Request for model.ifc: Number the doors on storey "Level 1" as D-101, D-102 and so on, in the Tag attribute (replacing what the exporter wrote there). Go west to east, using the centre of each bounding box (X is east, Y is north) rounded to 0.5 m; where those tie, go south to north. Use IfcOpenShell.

First a look at what the model holds.

```python
import ifcopenshell
import ifcopenshell.util.element
import ifcopenshell.util.placement

model = ifcopenshell.open("model.ifc")
print(model.schema)
storey = next(s for s in model.by_type("IfcBuildingStorey") if s.Name == "Level 1")
doors = [e for e in ifcopenshell.util.element.get_decomposition(storey) if e.is_a("IfcDoor")]
for e in sorted(doors, key=lambda e: e.id()):
    origin = ifcopenshell.util.placement.get_local_placement(e.ObjectPlacement)[:3, 3]
    print(e.id(), e.Tag, e.Name, origin.round(2) + 0.0, sep=" | ")
```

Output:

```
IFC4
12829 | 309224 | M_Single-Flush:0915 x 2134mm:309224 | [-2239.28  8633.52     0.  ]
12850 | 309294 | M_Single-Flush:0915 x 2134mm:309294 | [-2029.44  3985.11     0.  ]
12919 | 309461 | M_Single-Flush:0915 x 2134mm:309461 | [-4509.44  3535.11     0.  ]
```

```python
import ifcopenshell
import ifcopenshell.geom
import ifcopenshell.util.element
import ifcopenshell.util.shape

model = ifcopenshell.open("model.ifc")
settings = ifcopenshell.geom.settings()
settings.set("use-world-coords", True)


def centre(element):
    shape = ifcopenshell.geom.create_shape(settings, element)
    return ifcopenshell.util.shape.get_bbox_centroid(shape.geometry)


storey = next(s for s in model.by_type("IfcBuildingStorey") if s.Name == "Level 1")
doors = [e for e in ifcopenshell.util.element.get_decomposition(storey) if e.is_a("IfcDoor")]

# Insertion points can sit at a corner or the storey origin, so sort by the geometry (in metres).
centres = {e: centre(e) for e in doors}
doors.sort(key=lambda e: (round(centres[e][0] / 0.5), centres[e][1]))

for i, e in enumerate(doors, start=1):
    number = f"D-1{i:02d}"
    e.Tag = number
    print(e.id(), number)

model.write("model_v2.ifc")
```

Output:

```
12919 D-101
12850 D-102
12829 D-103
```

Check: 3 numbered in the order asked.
